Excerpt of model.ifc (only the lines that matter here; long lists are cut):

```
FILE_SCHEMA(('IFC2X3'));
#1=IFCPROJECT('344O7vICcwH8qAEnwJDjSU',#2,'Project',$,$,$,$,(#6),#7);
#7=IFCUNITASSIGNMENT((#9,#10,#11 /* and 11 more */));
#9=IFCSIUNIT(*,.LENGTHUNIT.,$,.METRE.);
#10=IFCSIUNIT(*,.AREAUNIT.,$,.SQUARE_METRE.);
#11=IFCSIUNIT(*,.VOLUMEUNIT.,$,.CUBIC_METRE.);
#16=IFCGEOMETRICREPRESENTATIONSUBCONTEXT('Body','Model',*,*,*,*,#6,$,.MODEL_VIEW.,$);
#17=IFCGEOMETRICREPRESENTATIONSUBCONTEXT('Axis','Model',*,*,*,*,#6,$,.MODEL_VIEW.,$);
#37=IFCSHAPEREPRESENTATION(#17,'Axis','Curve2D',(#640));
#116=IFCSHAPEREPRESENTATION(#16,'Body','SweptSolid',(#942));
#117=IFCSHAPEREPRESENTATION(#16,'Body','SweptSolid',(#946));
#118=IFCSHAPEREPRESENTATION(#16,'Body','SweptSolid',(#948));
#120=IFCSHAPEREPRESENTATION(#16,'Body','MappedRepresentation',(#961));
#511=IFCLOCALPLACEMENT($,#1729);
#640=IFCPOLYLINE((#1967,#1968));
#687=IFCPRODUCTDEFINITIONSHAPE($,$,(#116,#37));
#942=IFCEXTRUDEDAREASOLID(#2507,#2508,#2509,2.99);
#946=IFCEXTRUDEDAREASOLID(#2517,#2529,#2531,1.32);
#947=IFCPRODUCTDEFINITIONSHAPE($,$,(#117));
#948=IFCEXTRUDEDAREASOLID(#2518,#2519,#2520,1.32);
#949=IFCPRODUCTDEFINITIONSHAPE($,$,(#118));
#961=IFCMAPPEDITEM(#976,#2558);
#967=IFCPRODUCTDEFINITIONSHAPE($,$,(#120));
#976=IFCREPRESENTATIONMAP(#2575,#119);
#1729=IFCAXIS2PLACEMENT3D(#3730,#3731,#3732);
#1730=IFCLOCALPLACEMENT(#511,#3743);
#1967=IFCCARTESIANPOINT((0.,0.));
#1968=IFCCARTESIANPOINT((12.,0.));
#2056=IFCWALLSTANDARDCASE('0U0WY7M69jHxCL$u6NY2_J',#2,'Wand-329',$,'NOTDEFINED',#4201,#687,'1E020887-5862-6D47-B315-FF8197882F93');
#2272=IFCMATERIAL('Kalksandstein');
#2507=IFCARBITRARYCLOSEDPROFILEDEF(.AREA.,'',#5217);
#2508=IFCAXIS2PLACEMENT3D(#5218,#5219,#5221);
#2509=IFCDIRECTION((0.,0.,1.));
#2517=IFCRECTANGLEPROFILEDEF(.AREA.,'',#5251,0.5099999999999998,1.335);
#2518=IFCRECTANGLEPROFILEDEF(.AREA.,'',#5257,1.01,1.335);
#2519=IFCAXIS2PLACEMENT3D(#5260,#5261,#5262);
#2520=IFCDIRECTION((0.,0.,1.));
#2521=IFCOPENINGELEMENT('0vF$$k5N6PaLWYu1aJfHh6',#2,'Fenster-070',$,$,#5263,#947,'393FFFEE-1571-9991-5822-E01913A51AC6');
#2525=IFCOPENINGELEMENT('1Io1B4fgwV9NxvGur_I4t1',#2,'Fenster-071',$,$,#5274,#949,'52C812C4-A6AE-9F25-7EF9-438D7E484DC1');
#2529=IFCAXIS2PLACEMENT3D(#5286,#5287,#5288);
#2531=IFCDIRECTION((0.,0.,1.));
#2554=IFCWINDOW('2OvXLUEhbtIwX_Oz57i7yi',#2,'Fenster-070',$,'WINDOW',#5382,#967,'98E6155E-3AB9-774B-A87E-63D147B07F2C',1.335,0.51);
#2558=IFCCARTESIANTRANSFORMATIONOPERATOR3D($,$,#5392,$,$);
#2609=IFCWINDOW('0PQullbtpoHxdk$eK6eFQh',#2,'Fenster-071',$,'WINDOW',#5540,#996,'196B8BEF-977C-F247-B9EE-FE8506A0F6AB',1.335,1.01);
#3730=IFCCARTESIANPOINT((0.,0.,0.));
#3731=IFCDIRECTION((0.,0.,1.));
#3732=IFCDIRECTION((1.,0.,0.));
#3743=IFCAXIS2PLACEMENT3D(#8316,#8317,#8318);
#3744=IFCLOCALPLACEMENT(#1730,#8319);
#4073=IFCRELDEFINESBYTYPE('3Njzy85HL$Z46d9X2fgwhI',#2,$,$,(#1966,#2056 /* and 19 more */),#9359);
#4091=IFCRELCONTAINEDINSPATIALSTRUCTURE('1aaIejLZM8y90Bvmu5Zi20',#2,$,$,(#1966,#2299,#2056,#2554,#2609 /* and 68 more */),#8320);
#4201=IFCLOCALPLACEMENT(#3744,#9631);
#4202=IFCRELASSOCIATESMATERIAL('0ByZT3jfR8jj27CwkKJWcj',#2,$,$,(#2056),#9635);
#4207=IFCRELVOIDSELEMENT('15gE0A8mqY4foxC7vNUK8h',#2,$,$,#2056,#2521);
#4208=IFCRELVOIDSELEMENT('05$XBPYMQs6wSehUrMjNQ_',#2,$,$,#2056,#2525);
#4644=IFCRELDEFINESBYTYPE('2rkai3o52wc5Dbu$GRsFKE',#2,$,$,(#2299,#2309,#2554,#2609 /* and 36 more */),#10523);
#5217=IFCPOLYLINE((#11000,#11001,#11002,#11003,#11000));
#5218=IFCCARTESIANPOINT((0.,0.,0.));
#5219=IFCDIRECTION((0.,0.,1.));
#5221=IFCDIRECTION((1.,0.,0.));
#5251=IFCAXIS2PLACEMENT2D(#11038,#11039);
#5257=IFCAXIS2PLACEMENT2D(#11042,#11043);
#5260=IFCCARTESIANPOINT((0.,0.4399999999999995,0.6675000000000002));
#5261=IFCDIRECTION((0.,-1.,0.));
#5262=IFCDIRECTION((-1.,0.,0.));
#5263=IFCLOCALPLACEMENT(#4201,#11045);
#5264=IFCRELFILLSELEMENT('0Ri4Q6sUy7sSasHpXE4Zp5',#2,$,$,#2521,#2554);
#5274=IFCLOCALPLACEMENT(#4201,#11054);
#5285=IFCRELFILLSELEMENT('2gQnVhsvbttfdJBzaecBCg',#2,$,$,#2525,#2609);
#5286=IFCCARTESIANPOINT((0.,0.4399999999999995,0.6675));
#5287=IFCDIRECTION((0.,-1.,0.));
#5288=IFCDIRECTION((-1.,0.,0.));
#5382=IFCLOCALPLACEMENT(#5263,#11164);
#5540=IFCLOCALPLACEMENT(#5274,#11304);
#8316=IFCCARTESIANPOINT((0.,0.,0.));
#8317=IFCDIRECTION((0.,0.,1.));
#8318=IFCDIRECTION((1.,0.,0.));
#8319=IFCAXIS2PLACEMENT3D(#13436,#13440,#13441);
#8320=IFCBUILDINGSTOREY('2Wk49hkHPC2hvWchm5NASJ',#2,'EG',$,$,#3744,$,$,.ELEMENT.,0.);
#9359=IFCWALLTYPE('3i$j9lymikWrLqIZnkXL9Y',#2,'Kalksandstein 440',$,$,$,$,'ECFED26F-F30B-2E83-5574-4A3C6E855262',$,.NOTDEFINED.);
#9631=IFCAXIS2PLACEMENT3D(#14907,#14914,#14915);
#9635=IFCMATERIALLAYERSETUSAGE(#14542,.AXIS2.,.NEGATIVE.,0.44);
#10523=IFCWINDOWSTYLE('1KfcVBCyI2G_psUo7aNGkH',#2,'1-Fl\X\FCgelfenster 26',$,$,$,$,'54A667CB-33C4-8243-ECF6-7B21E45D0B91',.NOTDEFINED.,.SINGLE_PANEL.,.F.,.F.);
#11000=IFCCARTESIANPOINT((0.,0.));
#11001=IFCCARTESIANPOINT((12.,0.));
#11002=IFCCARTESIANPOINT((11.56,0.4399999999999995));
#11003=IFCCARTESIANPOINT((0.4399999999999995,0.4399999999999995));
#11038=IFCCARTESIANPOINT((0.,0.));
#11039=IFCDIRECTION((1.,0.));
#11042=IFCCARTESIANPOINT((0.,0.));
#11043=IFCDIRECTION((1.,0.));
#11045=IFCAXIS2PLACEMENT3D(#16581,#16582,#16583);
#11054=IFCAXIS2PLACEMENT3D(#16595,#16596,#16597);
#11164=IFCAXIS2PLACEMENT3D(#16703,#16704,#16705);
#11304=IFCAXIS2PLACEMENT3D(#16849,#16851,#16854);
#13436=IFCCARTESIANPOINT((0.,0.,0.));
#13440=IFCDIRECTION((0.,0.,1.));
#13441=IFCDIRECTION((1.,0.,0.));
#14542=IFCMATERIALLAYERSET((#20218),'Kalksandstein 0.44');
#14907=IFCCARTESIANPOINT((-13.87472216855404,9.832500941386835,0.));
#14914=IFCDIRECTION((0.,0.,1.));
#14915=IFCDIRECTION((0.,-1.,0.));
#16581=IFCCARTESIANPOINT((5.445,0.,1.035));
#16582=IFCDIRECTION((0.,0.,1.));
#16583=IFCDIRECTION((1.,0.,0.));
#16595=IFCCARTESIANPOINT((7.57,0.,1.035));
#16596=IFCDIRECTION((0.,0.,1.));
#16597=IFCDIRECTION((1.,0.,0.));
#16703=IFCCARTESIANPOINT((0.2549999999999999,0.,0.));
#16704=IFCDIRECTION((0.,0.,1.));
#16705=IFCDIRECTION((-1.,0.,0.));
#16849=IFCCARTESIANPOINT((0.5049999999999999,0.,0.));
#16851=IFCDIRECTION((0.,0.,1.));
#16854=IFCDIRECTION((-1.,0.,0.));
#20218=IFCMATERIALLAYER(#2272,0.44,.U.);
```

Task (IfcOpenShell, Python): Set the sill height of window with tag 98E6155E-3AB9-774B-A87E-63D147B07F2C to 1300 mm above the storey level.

```python
import numpy as np
import ifcopenshell
import ifcopenshell.api.geometry
import ifcopenshell.geom
import ifcopenshell.util.element
import ifcopenshell.util.placement
import ifcopenshell.util.shape
import ifcopenshell.util.unit

model = ifcopenshell.open("model.ifc")
unit_scale = ifcopenshell.util.unit.calculate_unit_scale(model)

window = model.by_guid("2OvXLUEhbtIwX_Oz57i7yi")
opening = window.FillsVoids[0].RelatingOpeningElement
storey = ifcopenshell.util.element.get_container(window, ifc_class="IfcBuildingStorey")
level = ifcopenshell.util.placement.get_local_placement(storey.ObjectPlacement)[2, 3]

# The opening's origin need not be at the sill, so measure its lowest point.
shape = ifcopenshell.geom.create_shape(ifcopenshell.geom.settings(), opening)
bottom = ifcopenshell.util.shape.get_shape_bottom_elevation(shape, shape.geometry) / unit_scale
dz = level + 1.3 - bottom

shift = np.array([0.0, 0.0, dz])
# The window is placed relative to its opening, so it follows when the opening moves.
matrix = ifcopenshell.util.placement.get_local_placement(opening.ObjectPlacement)
matrix[:3, 3] += shift
ifcopenshell.api.geometry.edit_object_placement(
    model, product=opening, matrix=matrix, is_si=False, should_transform_children=True
)

print(f"moved by {dz * unit_scale:+.3f} m")

model.write("model_rev.ifc")
```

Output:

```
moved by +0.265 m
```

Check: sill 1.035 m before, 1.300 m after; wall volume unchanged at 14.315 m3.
